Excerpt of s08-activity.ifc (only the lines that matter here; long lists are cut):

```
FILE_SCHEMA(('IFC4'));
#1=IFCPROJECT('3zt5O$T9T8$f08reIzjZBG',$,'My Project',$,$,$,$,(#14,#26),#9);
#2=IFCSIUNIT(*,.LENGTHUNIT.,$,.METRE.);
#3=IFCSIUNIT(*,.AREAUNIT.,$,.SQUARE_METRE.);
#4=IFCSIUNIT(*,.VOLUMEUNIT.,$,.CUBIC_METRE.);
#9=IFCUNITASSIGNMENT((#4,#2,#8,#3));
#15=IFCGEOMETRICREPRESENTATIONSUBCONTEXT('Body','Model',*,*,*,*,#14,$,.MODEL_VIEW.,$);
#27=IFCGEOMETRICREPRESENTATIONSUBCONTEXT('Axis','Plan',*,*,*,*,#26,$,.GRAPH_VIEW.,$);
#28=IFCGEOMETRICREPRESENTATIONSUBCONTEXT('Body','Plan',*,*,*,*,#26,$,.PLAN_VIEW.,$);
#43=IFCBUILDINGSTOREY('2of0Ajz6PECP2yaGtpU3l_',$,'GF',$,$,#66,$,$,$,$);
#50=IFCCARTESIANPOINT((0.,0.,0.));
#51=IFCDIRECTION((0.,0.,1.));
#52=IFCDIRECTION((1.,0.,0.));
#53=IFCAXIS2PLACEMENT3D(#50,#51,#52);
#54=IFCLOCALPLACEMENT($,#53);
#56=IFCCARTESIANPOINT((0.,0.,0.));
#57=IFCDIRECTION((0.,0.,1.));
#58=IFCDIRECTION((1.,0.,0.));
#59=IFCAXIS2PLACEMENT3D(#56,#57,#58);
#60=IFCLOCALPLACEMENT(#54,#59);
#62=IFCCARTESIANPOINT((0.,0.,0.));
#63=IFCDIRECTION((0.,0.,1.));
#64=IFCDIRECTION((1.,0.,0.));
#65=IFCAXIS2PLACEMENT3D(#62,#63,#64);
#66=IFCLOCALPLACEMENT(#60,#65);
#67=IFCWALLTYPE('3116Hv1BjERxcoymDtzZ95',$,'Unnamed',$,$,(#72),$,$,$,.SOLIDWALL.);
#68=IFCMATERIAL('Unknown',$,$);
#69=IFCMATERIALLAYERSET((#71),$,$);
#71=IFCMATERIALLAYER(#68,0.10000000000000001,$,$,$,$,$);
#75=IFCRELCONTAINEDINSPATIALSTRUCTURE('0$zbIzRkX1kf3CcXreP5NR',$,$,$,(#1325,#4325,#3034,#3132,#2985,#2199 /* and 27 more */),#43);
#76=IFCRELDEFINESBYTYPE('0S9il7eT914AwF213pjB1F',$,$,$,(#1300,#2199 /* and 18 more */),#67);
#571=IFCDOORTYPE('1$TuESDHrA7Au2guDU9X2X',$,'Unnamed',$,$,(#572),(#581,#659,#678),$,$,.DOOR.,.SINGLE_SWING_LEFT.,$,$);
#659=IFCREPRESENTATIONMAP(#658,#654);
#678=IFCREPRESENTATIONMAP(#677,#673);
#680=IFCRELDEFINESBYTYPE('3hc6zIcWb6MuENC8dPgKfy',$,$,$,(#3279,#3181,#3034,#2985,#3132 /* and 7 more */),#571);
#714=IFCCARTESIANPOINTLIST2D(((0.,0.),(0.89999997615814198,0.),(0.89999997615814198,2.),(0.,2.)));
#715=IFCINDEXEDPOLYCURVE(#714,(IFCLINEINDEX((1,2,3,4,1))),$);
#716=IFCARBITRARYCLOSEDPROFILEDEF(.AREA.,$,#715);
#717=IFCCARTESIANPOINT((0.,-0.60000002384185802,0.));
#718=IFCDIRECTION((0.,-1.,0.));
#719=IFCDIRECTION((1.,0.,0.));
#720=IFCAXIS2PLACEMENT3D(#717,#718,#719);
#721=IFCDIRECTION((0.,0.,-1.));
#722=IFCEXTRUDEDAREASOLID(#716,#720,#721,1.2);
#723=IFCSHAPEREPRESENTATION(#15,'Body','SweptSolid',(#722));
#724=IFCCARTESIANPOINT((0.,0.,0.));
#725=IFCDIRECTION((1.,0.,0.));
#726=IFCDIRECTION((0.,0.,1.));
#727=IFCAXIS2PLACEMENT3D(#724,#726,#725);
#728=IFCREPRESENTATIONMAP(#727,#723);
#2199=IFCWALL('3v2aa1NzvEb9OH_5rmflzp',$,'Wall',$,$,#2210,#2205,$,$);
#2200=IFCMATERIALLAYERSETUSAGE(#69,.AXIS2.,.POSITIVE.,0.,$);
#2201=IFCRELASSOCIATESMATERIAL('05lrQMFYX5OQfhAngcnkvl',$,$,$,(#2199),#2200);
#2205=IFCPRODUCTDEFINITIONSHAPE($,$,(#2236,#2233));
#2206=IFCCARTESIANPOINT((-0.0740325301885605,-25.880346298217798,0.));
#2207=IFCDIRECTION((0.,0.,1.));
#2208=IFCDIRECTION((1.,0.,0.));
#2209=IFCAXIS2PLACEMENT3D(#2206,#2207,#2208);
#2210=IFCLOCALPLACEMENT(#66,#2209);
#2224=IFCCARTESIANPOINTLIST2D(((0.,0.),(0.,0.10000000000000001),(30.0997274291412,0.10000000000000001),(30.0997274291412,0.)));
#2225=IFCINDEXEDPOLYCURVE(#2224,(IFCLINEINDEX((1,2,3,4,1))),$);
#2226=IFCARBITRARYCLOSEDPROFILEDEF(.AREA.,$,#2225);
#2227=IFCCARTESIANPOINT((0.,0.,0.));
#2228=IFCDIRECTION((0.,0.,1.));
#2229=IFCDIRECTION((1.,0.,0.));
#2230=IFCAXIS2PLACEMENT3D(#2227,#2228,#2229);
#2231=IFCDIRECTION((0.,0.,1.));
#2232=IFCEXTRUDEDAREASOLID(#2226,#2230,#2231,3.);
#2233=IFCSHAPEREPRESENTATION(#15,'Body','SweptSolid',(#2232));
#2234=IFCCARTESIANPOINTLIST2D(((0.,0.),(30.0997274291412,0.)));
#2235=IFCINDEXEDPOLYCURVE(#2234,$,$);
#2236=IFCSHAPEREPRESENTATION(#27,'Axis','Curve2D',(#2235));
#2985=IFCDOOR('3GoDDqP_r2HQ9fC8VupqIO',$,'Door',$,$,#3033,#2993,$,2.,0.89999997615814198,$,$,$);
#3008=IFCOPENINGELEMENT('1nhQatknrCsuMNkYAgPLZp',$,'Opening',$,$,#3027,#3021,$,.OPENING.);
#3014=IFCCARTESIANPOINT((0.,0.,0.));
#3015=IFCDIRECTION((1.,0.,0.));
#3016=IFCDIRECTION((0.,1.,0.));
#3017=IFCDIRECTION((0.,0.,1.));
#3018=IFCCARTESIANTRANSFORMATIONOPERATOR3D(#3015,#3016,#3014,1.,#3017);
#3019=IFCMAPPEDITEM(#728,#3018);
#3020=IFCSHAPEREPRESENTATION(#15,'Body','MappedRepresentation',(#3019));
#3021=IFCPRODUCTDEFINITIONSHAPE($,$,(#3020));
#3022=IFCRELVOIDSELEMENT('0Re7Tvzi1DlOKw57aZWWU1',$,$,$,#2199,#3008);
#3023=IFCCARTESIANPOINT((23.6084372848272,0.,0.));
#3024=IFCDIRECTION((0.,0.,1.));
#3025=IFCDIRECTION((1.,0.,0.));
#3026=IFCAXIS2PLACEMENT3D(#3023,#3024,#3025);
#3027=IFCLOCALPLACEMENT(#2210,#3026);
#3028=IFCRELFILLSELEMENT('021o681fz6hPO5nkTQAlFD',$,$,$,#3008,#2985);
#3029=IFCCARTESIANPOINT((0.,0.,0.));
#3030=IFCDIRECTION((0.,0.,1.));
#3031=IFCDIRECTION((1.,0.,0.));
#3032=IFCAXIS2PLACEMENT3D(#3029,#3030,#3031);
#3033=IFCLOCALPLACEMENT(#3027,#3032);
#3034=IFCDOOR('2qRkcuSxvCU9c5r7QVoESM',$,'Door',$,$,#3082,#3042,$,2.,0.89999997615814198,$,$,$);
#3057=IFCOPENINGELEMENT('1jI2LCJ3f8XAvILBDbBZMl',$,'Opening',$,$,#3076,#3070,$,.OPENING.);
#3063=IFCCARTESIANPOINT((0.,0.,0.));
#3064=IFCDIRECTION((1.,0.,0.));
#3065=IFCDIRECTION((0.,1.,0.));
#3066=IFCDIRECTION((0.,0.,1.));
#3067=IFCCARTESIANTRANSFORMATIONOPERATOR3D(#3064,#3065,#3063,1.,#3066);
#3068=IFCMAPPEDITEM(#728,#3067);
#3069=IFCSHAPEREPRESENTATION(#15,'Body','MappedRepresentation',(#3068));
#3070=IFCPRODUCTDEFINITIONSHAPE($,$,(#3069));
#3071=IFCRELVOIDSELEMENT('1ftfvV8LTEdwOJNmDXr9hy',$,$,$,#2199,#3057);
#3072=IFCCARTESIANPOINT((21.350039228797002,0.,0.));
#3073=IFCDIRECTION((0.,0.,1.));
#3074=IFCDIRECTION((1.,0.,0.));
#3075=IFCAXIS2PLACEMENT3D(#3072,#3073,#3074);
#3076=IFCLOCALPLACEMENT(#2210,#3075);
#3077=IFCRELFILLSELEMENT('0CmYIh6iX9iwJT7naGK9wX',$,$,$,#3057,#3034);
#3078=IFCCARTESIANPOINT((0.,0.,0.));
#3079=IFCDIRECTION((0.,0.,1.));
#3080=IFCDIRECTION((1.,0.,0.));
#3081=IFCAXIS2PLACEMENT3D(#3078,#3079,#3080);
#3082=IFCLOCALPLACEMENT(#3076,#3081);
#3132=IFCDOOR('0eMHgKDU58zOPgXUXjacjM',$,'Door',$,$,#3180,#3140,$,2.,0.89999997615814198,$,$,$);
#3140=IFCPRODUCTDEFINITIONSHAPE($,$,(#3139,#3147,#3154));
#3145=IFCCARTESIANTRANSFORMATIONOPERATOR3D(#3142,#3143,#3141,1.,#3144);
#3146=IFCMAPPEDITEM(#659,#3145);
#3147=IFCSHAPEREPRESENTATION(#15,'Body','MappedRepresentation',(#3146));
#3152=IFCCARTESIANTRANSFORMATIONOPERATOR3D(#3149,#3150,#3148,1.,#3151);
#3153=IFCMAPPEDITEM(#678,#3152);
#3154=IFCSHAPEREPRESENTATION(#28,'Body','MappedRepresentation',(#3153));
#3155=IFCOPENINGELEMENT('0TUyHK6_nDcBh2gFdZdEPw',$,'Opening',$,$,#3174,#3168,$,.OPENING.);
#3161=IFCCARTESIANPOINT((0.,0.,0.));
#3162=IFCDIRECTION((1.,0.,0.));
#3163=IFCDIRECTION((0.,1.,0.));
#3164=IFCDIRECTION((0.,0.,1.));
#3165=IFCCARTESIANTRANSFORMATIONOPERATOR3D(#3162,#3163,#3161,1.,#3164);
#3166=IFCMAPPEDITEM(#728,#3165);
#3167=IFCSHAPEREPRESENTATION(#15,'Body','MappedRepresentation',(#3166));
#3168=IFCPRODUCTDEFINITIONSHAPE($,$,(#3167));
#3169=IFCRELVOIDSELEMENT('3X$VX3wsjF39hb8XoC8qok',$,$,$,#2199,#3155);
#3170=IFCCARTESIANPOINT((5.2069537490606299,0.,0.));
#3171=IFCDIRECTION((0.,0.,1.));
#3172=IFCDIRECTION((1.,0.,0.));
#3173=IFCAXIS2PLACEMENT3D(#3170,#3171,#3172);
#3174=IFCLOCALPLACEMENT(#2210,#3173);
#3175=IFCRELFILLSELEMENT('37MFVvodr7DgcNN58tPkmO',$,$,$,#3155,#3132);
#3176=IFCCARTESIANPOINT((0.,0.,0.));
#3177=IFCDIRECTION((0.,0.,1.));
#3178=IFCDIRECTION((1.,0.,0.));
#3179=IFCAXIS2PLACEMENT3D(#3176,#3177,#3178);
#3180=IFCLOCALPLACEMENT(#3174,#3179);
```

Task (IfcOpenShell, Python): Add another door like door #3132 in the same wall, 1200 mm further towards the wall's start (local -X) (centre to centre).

```python
import ifcopenshell
import ifcopenshell.api.feature
import ifcopenshell.api.geometry
import ifcopenshell.api.root
import ifcopenshell.geom
import ifcopenshell.util.element
import ifcopenshell.util.placement
import ifcopenshell.util.shape
import ifcopenshell.util.unit

model = ifcopenshell.open("s08-activity.ifc")
unit_scale = ifcopenshell.util.unit.calculate_unit_scale(model)
settings = ifcopenshell.geom.settings()


def volume(element):
    """Net volume in cubic metres, openings subtracted."""
    shape = ifcopenshell.geom.create_shape(settings, element)
    return ifcopenshell.util.shape.get_volume(shape.geometry)


door = model.by_id(3132)
opening = door.FillsVoids[0].RelatingOpeningElement
wall = opening.VoidsElements[0].RelatingBuildingElement
before = volume(wall)
shift = ifcopenshell.util.placement.get_local_placement(wall.ObjectPlacement)[:3, 0] * -1.2 / unit_scale

# copy_class copies the void relationship, type, container and properties, but no geometry.
new_opening = ifcopenshell.api.root.copy_class(model, product=opening)
new_opening.Representation = ifcopenshell.util.element.copy_deep(
    model, opening.Representation, exclude=["IfcGeometricRepresentationContext", "IfcRepresentationMap"]
)
new_door = ifcopenshell.api.root.copy_class(model, product=door)
new_door.Representation = ifcopenshell.util.element.copy_deep(
    model, door.Representation, exclude=["IfcGeometricRepresentationContext", "IfcRepresentationMap"]
)
ifcopenshell.api.feature.add_filling(model, opening=new_opening, element=new_door)

for old, new in ((opening, new_opening), (door, new_door)):
    matrix = ifcopenshell.util.placement.get_local_placement(old.ObjectPlacement)
    matrix[:3, 3] += shift
    ifcopenshell.api.geometry.edit_object_placement(model, product=new, matrix=matrix, is_si=False)

after = volume(wall)

print(f"wall volume {before:.3f} -> {after:.3f} m3")

model.write("s08-activity_edited.ifc")
```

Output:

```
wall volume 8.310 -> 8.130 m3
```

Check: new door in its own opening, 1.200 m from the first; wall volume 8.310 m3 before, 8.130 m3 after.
